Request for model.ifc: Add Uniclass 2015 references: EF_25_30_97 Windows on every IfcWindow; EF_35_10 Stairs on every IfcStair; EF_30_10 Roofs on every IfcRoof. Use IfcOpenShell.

First a look at what the model holds.

```python
import ifcopenshell

model = ifcopenshell.open("model.ifc")
print(model.schema)
print("classifications:", [c.Name for c in model.by_type("IfcClassification")])
for ifc_class in ("IfcDoor", "IfcRoof", "IfcStair", "IfcWall", "IfcWindow"):
    print(ifc_class, len(model.by_type(ifc_class)))
```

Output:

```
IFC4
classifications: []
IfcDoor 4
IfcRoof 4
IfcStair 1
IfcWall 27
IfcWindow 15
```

```python
import ifcopenshell
import ifcopenshell.api.classification

model = ifcopenshell.open("model.ifc")

system = ifcopenshell.api.classification.add_classification(model, classification="Uniclass 2015")

codes = {
    "IfcWindow": ("EF_25_30_97", "Windows"),
    "IfcStair": ("EF_35_10", "Stairs"),
    "IfcRoof": ("EF_30_10", "Roofs"),
}
for ifc_class, (code, name) in codes.items():
    products = model.by_type(ifc_class)
    ifcopenshell.api.classification.add_reference(
        model, products=products, classification=system, identification=code, name=name
    )
    print(code, len(products))

model.write("model_v2.ifc")
```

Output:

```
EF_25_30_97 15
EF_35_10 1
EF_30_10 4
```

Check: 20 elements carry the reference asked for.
